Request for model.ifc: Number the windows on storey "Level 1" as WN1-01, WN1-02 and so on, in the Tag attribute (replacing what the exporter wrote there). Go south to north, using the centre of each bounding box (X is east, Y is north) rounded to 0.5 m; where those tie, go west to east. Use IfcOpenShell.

First a look at what the model holds.

```python
import ifcopenshell
import ifcopenshell.util.element
import ifcopenshell.util.placement

model = ifcopenshell.open("model.ifc")
print(model.schema)
storey = next(s for s in model.by_type("IfcBuildingStorey") if s.Name == "Level 1")
windows = [e for e in ifcopenshell.util.element.get_decomposition(storey) if e.is_a("IfcWindow")]
for e in sorted(windows, key=lambda e: e.id()):
    origin = ifcopenshell.util.placement.get_local_placement(e.ObjectPlacement)[:3, 3]
    print(e.id(), e.Tag, e.Name, origin.round(2) + 0.0, sep=" | ")
```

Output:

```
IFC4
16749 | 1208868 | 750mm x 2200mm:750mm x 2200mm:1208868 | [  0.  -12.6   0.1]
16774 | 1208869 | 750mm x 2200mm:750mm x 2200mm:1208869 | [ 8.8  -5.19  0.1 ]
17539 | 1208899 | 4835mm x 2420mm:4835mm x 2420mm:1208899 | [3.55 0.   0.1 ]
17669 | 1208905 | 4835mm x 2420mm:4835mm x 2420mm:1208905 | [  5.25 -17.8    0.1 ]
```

```python
import ifcopenshell
import ifcopenshell.geom
import ifcopenshell.util.element
import ifcopenshell.util.shape

model = ifcopenshell.open("model.ifc")
settings = ifcopenshell.geom.settings()
settings.set("use-world-coords", True)


def centre(element):
    shape = ifcopenshell.geom.create_shape(settings, element)
    return ifcopenshell.util.shape.get_bbox_centroid(shape.geometry)


storey = next(s for s in model.by_type("IfcBuildingStorey") if s.Name == "Level 1")
windows = [e for e in ifcopenshell.util.element.get_decomposition(storey) if e.is_a("IfcWindow")]

# Insertion points can sit at a corner or the storey origin, so sort by the geometry (in metres).
centres = {e: centre(e) for e in windows}
windows.sort(key=lambda e: (round(centres[e][1] / 0.5), centres[e][0]))

for i, e in enumerate(windows, start=1):
    number = f"WN1-{i:02d}"
    e.Tag = number
    print(e.id(), number)

model.write("model_edited.ifc")
```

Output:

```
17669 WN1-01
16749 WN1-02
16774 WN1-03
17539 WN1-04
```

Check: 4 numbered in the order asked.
